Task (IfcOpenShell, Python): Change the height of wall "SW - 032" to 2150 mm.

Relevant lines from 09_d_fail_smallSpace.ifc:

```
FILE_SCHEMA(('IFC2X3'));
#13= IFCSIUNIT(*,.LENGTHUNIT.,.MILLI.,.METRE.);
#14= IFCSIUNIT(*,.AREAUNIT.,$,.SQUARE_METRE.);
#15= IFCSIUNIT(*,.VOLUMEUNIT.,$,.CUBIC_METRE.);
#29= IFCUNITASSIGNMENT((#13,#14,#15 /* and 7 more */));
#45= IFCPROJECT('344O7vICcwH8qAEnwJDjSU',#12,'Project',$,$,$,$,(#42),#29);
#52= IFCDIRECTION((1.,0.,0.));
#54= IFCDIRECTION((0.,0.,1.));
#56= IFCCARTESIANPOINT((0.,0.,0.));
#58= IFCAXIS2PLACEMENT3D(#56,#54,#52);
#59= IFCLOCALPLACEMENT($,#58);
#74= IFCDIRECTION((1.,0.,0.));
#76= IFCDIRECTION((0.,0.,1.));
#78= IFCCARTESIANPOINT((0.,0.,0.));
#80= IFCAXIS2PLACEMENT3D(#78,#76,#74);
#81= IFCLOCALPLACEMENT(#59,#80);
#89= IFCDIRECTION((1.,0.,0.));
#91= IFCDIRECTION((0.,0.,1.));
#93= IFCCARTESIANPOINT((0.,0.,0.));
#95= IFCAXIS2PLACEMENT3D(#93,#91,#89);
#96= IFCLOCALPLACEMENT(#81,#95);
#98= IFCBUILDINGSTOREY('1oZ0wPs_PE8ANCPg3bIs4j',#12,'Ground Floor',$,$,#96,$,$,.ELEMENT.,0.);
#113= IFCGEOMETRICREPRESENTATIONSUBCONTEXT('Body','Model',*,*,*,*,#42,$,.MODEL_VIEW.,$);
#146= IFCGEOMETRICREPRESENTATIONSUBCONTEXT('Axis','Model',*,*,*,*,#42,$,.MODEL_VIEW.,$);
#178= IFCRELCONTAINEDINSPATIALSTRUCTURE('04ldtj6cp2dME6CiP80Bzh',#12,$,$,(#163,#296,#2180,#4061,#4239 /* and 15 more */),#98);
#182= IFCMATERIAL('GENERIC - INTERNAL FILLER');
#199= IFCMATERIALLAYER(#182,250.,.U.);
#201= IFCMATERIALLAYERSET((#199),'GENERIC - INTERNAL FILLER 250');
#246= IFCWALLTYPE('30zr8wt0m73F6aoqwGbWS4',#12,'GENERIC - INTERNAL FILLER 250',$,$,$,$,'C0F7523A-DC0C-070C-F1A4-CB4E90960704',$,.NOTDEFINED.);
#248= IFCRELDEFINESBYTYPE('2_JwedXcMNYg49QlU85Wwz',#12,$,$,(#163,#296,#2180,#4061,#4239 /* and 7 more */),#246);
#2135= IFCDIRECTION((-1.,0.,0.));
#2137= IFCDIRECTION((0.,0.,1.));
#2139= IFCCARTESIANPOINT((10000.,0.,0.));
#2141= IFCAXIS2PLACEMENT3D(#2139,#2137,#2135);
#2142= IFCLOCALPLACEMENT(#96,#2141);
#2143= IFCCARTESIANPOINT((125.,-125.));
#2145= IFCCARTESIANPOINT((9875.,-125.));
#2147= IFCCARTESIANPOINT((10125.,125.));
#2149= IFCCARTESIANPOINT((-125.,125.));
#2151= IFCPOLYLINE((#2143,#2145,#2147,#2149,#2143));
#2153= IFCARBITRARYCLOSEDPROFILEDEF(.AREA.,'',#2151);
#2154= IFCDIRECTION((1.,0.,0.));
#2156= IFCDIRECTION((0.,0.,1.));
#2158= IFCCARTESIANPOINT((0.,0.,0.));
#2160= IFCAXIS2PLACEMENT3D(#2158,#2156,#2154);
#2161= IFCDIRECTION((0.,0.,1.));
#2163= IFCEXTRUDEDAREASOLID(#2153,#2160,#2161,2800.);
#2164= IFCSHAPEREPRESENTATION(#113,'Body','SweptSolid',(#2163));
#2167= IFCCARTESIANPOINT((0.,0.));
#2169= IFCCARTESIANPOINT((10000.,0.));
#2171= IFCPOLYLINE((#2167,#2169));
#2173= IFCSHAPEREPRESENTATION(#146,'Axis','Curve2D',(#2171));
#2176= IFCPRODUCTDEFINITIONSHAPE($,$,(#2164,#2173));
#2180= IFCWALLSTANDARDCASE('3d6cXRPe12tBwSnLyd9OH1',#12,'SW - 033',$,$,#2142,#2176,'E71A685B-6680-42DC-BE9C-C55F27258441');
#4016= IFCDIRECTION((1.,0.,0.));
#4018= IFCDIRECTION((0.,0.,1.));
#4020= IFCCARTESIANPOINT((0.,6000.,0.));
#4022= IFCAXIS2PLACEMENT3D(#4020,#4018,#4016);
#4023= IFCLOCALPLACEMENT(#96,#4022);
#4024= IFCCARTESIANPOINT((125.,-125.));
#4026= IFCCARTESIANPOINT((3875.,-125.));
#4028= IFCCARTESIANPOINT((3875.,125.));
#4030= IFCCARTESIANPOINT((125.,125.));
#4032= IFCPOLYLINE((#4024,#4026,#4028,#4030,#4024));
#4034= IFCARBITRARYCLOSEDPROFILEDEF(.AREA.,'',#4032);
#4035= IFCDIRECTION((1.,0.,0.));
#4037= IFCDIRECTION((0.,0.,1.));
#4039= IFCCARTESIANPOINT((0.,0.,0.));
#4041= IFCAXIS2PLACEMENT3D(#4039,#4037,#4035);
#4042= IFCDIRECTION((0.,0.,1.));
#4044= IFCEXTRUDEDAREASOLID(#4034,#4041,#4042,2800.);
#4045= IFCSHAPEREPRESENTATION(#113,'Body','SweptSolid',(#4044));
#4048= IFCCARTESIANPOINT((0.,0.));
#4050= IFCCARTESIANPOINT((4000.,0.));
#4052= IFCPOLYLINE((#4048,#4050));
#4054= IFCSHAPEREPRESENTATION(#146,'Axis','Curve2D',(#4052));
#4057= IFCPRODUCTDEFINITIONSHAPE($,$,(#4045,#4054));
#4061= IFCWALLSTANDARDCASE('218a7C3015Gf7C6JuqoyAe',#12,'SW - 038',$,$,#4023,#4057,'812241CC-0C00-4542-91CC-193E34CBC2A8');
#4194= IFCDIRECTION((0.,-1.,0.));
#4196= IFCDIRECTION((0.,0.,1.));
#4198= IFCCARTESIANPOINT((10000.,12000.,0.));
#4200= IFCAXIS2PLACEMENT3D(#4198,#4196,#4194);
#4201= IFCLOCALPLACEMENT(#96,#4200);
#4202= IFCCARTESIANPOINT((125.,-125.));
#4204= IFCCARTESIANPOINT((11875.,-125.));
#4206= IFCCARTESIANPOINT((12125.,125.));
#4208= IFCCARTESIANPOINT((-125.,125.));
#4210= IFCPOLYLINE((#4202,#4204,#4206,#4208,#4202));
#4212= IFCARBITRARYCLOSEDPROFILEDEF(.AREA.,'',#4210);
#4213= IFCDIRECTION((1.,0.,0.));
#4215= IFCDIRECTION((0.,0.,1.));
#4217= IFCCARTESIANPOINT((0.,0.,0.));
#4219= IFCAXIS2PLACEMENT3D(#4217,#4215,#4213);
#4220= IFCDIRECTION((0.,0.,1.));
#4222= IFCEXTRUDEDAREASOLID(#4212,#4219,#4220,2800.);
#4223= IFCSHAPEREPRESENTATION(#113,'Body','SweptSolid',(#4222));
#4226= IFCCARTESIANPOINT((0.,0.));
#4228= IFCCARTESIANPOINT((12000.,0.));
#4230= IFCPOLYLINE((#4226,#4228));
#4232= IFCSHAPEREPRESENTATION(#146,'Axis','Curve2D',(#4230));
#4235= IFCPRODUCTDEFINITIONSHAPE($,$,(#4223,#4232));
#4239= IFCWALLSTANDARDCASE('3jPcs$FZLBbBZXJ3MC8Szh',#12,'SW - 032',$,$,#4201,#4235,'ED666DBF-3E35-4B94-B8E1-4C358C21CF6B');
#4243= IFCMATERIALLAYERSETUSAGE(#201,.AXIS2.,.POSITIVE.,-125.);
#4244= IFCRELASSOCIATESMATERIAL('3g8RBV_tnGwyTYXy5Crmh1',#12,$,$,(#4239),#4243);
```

```python
import ifcopenshell
import ifcopenshell.geom
import ifcopenshell.util.representation
import ifcopenshell.util.shape
import ifcopenshell.util.unit

model = ifcopenshell.open("09_d_fail_smallSpace.ifc")
unit_scale = ifcopenshell.util.unit.calculate_unit_scale(model)
settings = ifcopenshell.geom.settings()


def volume(element):
    """Net volume in cubic metres, openings subtracted."""
    shape = ifcopenshell.geom.create_shape(settings, element)
    return ifcopenshell.util.shape.get_volume(shape.geometry)


wall = model.by_id(4239)
before = volume(wall)

body = ifcopenshell.util.representation.get_representation(wall, "Model", "Body")
solid = body.Items[0]
old_height = solid.Depth
solid.Depth = 2.15 / unit_scale
after = volume(wall)

print(f"height {old_height:g} -> {solid.Depth:g}, volume {before:.3f} -> {after:.3f} m3")

model.write("09_d_fail_smallSpace_edited.ifc")
```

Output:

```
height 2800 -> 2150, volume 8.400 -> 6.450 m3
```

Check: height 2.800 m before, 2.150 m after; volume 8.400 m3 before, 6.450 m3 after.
